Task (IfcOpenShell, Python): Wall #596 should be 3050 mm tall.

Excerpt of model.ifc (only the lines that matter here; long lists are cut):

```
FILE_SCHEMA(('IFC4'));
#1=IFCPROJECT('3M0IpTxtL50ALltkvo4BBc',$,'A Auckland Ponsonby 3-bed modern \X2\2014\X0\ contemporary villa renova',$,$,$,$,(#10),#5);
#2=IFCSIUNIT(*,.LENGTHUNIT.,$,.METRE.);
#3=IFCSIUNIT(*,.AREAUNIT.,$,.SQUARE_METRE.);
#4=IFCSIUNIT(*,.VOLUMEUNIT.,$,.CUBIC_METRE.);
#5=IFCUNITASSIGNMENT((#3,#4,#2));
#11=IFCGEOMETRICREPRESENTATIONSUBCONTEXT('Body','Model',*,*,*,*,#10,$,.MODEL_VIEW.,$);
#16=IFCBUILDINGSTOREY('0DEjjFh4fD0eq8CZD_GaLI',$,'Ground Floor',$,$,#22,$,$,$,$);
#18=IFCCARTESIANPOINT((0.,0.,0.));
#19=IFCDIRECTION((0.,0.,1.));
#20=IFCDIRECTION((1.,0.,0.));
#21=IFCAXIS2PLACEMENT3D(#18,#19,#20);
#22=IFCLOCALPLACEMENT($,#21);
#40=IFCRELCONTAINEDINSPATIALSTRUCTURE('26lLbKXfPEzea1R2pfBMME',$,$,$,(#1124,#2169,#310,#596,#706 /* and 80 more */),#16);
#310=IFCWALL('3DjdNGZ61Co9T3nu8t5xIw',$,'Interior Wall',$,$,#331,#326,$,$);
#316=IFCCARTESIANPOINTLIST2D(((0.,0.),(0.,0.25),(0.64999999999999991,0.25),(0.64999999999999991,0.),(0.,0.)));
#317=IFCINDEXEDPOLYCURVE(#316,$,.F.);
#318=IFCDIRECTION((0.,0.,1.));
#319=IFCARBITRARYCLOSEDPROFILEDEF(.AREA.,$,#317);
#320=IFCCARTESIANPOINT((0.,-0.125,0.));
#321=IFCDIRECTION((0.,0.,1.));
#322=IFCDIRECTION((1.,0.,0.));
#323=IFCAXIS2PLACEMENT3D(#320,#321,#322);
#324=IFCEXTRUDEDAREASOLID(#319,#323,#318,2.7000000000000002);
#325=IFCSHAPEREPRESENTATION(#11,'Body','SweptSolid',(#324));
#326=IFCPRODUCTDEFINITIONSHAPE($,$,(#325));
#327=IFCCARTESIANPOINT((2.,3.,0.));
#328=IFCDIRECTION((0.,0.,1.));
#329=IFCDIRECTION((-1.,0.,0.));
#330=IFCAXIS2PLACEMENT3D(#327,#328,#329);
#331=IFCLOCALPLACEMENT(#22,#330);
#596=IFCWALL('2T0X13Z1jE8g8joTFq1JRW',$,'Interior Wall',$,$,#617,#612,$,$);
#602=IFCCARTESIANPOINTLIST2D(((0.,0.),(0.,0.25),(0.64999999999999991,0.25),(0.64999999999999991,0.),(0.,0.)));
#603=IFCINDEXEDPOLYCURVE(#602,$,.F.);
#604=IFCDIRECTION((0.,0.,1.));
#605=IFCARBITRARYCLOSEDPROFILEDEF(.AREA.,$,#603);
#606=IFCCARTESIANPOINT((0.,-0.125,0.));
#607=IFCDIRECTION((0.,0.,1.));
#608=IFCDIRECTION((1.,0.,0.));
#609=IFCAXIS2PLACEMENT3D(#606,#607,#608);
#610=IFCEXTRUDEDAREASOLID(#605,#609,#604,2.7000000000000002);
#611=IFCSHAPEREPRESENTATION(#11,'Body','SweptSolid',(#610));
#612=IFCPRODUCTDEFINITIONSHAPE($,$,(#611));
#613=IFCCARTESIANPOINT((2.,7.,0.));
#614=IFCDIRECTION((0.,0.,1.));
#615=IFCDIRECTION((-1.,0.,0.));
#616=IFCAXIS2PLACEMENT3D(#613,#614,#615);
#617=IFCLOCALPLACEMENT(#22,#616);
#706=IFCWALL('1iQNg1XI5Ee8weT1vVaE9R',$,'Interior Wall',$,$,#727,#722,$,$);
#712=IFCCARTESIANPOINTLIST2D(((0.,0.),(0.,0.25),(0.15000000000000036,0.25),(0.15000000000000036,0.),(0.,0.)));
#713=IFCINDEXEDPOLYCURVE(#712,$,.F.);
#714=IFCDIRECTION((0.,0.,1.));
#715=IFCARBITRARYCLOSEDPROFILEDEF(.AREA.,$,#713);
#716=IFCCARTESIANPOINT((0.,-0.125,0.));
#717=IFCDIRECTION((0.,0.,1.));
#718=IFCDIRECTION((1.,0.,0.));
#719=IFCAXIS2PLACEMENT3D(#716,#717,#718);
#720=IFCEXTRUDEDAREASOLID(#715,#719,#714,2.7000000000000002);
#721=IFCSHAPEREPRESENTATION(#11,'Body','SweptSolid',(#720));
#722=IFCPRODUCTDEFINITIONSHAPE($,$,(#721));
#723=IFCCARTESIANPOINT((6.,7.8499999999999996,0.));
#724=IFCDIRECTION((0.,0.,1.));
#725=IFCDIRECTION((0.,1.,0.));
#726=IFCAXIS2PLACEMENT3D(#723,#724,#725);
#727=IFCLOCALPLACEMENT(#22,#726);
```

```python
import ifcopenshell
import ifcopenshell.geom
import ifcopenshell.util.representation
import ifcopenshell.util.shape
import ifcopenshell.util.unit

model = ifcopenshell.open("model.ifc")
unit_scale = ifcopenshell.util.unit.calculate_unit_scale(model)
settings = ifcopenshell.geom.settings()


def volume(element):
    """Net volume in cubic metres, openings subtracted."""
    shape = ifcopenshell.geom.create_shape(settings, element)
    return ifcopenshell.util.shape.get_volume(shape.geometry)


wall = model.by_id(596)
before = volume(wall)

body = ifcopenshell.util.representation.get_representation(wall, "Model", "Body")
solid = body.Items[0]
old_height = solid.Depth
solid.Depth = 3.05 / unit_scale
after = volume(wall)

print(f"height {old_height:g} -> {solid.Depth:g}, volume {before:.3f} -> {after:.3f} m3")

model.write("model_edited.ifc")
```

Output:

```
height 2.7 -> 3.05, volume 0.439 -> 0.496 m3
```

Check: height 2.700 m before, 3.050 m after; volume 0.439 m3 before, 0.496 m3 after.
